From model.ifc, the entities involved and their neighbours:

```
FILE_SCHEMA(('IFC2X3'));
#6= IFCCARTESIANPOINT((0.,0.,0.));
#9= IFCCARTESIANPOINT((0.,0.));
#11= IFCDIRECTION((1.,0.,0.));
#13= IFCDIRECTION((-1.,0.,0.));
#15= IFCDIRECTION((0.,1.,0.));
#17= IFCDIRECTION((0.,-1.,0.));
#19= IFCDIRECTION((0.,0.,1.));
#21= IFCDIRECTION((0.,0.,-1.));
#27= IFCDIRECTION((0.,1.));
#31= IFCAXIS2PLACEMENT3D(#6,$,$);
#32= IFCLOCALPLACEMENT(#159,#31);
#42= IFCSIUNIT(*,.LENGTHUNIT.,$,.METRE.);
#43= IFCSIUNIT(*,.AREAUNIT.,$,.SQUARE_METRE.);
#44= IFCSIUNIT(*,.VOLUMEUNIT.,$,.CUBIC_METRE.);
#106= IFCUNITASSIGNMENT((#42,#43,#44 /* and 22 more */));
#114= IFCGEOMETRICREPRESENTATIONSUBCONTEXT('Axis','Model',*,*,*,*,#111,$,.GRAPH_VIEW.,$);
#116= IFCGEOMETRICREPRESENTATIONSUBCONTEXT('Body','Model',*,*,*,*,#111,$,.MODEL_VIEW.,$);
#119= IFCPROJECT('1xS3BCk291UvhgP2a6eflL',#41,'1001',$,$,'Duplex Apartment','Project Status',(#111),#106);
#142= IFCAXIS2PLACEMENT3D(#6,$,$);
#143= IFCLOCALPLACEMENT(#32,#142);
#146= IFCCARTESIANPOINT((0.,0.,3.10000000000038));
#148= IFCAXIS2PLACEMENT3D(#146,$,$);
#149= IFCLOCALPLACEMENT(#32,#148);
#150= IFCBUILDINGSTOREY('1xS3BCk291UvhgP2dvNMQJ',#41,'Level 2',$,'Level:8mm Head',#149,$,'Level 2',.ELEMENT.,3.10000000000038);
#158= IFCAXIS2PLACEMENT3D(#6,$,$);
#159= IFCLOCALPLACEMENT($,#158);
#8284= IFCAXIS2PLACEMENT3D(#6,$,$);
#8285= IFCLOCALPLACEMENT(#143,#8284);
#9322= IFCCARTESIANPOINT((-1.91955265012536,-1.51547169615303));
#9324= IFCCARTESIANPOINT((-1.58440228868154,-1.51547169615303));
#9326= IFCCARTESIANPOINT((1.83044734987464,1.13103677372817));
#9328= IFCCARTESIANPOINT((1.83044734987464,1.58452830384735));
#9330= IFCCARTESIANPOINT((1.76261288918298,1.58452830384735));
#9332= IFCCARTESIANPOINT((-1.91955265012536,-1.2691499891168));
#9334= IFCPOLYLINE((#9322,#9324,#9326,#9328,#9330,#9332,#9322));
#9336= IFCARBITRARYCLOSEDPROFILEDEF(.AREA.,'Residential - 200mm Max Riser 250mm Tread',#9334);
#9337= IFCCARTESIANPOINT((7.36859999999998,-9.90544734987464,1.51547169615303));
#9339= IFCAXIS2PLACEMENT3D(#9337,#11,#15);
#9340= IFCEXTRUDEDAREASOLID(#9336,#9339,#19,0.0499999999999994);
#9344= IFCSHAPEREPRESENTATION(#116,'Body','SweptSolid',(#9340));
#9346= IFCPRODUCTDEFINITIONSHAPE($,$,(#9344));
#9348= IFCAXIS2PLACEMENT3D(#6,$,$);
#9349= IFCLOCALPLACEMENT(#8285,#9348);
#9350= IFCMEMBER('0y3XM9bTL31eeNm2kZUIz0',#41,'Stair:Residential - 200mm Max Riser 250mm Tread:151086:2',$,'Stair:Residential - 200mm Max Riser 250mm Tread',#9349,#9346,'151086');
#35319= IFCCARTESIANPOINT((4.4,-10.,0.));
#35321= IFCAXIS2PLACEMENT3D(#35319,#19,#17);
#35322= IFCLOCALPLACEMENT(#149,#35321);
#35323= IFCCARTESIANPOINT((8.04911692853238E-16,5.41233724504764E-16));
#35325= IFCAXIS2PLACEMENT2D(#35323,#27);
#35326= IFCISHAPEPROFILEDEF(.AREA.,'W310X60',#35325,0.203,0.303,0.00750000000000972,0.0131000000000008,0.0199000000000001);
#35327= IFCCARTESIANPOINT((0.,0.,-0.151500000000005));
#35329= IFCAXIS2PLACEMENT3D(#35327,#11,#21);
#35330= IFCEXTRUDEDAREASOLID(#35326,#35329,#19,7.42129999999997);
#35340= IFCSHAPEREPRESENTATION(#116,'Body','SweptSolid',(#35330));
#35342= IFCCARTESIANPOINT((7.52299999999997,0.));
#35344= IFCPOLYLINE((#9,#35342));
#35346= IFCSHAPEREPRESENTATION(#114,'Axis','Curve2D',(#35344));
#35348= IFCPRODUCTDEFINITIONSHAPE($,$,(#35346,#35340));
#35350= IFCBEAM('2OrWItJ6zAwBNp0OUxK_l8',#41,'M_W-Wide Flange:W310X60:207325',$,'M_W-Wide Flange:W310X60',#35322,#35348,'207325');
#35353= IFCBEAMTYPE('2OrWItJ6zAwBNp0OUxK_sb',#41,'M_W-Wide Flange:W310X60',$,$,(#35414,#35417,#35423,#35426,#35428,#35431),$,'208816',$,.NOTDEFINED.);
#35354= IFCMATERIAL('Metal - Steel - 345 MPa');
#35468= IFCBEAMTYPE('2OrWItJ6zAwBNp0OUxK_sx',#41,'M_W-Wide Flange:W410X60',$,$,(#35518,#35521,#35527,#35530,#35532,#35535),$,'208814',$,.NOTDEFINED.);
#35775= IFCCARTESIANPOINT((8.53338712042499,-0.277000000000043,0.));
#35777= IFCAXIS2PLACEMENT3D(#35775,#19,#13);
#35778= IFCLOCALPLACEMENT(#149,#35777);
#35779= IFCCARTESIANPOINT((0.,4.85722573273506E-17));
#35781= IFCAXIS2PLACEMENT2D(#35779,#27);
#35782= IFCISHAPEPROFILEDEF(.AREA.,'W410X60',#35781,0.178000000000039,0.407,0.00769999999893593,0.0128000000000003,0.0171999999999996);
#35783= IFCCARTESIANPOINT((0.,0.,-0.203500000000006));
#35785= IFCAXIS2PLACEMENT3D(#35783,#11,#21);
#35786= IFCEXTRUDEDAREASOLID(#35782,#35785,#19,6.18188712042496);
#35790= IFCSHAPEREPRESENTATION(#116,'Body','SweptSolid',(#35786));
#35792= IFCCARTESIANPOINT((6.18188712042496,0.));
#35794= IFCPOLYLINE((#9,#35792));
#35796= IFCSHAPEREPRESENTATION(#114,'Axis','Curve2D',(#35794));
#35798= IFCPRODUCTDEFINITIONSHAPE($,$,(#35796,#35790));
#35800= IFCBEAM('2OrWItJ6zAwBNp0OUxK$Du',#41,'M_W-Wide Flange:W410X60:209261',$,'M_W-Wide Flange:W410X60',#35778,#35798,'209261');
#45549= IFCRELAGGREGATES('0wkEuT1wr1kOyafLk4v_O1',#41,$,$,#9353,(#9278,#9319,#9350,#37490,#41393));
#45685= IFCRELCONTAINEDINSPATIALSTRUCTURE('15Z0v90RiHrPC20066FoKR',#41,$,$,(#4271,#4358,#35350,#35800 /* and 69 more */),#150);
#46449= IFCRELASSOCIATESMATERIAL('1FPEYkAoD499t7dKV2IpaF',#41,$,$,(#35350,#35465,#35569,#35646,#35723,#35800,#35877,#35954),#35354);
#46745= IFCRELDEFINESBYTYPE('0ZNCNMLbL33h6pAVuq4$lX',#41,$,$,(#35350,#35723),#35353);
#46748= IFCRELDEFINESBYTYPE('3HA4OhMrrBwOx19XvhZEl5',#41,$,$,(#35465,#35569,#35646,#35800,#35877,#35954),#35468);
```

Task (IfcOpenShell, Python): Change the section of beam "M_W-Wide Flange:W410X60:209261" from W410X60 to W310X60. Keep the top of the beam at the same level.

```python
import ifcopenshell
import ifcopenshell.api.type
import ifcopenshell.util.element
import ifcopenshell.util.representation

model = ifcopenshell.open("model.ifc")

member = model.by_id(35800)
source = next(p for p in model.by_type("IfcIShapeProfileDef") if p.ProfileName == "W310X60")

body = ifcopenshell.util.representation.get_representation(member, "Model", "Body")
solid = body.Items[0]
old_profile = solid.SweptArea

# Copy the section's sizes but keep this member's own profile position.
profile = ifcopenshell.util.element.copy(model, source)
# Profiles are centred, so shift by half the change in depth to hold the top.
shift = (old_profile.OverallDepth - profile.OverallDepth) / 2
x, y = old_profile.Position.Location.Coordinates
up = (-1.0, 0.0)  # upwards, in the solid's own plane
location = model.createIfcCartesianPoint((x + up[0] * shift, y + up[1] * shift))
profile.Position = model.createIfcAxis2Placement2D(location, old_profile.Position.RefDirection)
solid.SweptArea = profile
if not model.get_total_inverses(old_profile):
    ifcopenshell.util.element.remove_deep2(model, old_profile)

new_type = model.by_guid("2OrWItJ6zAwBNp0OUxK_sb")
ifcopenshell.api.type.assign_type(
    model, related_objects=[member], relating_type=new_type, should_map_representations=False
)
member.Name = member.Name.replace("W410X60", "W310X60")
member.ObjectType = "M_W-Wide Flange:W310X60"

print(solid.SweptArea)

model.write("model_updated.ifc")
```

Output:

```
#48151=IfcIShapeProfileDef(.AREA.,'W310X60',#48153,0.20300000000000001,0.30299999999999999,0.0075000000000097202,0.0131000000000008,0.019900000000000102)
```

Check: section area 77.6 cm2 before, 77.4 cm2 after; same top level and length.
